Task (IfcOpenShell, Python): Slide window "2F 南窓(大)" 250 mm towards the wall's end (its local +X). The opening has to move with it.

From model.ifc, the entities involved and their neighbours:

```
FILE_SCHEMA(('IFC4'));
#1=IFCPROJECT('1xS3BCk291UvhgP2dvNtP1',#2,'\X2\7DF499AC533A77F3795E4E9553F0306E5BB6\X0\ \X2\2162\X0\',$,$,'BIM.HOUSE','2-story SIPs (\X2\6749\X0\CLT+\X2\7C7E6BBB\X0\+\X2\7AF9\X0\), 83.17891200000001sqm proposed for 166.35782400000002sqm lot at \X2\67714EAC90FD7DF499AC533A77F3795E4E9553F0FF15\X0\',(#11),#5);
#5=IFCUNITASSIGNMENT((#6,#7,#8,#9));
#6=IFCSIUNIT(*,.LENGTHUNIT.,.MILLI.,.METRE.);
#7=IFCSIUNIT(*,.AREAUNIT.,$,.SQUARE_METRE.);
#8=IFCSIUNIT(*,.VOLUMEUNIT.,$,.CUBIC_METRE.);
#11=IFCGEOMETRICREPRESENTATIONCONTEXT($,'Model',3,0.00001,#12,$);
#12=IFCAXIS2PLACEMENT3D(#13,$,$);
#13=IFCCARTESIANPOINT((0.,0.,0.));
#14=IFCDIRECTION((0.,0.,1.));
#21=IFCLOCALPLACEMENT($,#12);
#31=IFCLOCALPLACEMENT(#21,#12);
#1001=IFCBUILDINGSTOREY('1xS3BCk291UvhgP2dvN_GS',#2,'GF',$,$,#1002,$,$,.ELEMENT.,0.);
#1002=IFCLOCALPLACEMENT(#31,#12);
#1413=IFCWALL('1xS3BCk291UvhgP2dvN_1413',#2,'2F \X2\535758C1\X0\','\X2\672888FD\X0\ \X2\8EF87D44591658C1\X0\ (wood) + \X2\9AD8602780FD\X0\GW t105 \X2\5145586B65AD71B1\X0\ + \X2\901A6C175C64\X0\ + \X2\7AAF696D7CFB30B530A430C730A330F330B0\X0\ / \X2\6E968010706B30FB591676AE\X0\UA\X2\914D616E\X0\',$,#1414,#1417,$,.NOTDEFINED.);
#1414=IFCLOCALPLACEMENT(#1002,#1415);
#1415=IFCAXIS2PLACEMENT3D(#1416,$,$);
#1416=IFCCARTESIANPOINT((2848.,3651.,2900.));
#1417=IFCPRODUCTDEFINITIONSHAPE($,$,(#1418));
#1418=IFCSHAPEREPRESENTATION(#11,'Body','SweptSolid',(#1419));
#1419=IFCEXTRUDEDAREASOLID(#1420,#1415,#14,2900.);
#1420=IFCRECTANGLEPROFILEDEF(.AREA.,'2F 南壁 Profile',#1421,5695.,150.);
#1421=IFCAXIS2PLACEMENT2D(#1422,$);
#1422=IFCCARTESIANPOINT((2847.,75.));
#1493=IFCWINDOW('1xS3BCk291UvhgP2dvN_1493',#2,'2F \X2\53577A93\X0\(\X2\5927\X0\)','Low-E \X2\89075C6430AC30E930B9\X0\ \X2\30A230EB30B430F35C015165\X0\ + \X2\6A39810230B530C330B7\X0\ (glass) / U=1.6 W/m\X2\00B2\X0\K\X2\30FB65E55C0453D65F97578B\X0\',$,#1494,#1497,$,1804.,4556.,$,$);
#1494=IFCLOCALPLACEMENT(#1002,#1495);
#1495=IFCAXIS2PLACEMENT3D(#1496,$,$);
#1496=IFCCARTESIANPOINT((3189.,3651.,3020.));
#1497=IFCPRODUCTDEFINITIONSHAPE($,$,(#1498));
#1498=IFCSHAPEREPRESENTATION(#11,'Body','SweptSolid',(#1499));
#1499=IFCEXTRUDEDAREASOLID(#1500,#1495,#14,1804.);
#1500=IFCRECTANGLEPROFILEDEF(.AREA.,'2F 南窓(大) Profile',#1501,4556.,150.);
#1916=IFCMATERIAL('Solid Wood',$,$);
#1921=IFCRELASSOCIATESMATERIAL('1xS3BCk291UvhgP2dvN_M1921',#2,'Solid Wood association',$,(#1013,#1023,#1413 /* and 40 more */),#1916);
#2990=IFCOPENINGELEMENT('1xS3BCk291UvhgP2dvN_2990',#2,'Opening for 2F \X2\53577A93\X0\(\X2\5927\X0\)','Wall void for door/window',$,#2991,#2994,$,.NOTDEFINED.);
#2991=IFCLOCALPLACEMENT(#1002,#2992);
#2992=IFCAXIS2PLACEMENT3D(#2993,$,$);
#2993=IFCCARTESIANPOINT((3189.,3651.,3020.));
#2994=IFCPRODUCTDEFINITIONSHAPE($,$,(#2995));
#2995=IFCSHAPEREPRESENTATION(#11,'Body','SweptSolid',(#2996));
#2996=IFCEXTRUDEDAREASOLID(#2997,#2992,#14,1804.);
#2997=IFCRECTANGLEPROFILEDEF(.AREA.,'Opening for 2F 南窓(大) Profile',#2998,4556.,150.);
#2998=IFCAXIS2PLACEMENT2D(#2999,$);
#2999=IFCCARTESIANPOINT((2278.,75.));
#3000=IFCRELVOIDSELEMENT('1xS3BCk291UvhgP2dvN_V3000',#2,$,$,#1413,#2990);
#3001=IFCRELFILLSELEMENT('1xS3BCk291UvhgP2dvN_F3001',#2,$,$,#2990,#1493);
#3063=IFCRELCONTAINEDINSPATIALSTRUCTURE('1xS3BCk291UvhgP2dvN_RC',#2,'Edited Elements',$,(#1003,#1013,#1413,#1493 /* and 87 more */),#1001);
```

```python
import ifcopenshell
import ifcopenshell.api.geometry
import ifcopenshell.util.placement
import ifcopenshell.util.unit

model = ifcopenshell.open("model.ifc")
unit_scale = ifcopenshell.util.unit.calculate_unit_scale(model)

window = model.by_id(1493)
opening = window.FillsVoids[0].RelatingOpeningElement
wall = opening.VoidsElements[0].RelatingBuildingElement

wall_matrix = ifcopenshell.util.placement.get_local_placement(wall.ObjectPlacement)
shift = wall_matrix[:3, 0] * 0.25 / unit_scale
before = ifcopenshell.util.placement.get_local_placement(window.ObjectPlacement)[:3, 3].copy()

# The window is not placed relative to its opening, so move both.
for product in (opening, window):
    matrix = ifcopenshell.util.placement.get_local_placement(product.ObjectPlacement)
    matrix[:3, 3] += shift
    ifcopenshell.api.geometry.edit_object_placement(model, product=product, matrix=matrix, is_si=False)

after = ifcopenshell.util.placement.get_local_placement(window.ObjectPlacement)[:3, 3]
print("window moved by", (after - before).round(3) + 0.0)

model.write("model_v2.ifc")
```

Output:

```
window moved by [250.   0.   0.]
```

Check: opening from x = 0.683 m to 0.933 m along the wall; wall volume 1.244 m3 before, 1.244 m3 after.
